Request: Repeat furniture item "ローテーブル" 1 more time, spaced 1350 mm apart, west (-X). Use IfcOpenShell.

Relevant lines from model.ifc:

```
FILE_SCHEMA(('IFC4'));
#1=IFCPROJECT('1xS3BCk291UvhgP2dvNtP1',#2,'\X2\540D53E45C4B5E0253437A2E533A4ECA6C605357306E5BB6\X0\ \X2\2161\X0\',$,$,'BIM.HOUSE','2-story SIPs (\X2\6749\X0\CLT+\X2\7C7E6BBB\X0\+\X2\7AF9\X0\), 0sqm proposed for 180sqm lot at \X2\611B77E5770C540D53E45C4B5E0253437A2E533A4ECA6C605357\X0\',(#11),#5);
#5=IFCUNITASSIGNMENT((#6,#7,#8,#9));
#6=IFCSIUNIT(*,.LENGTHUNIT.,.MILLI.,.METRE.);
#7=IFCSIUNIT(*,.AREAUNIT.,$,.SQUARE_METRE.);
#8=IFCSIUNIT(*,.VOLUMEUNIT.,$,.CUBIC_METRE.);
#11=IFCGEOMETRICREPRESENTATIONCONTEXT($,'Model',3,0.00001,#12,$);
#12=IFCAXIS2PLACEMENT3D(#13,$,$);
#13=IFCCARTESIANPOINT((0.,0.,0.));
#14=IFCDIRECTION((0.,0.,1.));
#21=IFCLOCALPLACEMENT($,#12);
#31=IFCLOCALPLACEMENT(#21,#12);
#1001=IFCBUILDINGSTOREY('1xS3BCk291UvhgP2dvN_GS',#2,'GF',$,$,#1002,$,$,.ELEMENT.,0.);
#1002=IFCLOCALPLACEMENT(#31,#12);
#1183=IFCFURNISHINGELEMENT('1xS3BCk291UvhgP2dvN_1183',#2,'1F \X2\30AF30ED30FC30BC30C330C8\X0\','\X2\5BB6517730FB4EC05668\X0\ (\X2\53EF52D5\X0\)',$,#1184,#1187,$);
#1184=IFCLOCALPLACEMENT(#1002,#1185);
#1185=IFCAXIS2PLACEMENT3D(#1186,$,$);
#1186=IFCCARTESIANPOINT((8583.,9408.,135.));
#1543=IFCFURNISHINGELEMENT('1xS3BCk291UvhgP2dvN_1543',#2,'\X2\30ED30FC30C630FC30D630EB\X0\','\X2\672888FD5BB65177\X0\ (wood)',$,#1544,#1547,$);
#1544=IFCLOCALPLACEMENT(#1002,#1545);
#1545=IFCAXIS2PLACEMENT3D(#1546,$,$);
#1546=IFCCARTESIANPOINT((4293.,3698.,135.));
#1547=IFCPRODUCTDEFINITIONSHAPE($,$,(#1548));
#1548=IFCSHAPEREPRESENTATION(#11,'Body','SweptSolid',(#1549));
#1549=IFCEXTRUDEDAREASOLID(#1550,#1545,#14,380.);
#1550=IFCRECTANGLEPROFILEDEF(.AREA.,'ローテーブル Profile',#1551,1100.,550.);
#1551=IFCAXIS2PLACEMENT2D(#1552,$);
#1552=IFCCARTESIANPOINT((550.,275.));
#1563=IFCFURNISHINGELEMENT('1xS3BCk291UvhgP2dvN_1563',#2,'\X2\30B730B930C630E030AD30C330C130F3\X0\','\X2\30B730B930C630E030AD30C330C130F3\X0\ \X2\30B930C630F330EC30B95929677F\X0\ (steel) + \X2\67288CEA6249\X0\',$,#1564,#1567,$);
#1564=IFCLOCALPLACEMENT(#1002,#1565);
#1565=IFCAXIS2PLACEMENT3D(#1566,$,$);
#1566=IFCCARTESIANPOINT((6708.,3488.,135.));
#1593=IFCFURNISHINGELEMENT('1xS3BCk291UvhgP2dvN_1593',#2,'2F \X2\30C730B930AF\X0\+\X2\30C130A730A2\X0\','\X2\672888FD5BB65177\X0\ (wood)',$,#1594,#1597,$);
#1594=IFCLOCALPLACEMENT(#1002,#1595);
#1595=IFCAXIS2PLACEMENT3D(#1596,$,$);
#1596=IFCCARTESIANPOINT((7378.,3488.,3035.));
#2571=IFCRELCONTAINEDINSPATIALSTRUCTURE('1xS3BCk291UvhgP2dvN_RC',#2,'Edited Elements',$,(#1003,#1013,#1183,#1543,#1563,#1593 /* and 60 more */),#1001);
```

```python
import numpy as np
import ifcopenshell
import ifcopenshell.api.geometry
import ifcopenshell.api.root
import ifcopenshell.util.element
import ifcopenshell.util.placement

model = ifcopenshell.open("model.ifc")


def reuse_history(source, copy):
    """copy_class also copies each property set's owner history, people and application; keep the originals."""
    for rel in copy.IsDefinedBy:
        if rel.is_a("IfcRelDefinesByProperties") and (history := rel.RelatingPropertyDefinition.OwnerHistory):
            rel.RelatingPropertyDefinition.OwnerHistory = source.OwnerHistory
            ifcopenshell.util.element.remove_deep2(model, history)


source = model.by_guid("1xS3BCk291UvhgP2dvN_1543")
base = ifcopenshell.util.placement.get_local_placement(source.ObjectPlacement)
step = np.array([-1.0, 0.0, 0.0]) * 1350.0

for i in range(1, 2):
    copy = ifcopenshell.api.root.copy_class(model, product=source)
    copy.Representation = ifcopenshell.util.element.copy_deep(
        model, source.Representation, exclude=["IfcGeometricRepresentationContext", "IfcRepresentationMap"]
    )
    reuse_history(source, copy)
    matrix = base.copy()
    matrix[:3, 3] += i * step
    print("added at", matrix[:3, 3].round(3) + 0.0)
    ifcopenshell.api.geometry.edit_object_placement(model, product=copy, matrix=matrix, is_si=False)

model.write("model_v2.ifc")
```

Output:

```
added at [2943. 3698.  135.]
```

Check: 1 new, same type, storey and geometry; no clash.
